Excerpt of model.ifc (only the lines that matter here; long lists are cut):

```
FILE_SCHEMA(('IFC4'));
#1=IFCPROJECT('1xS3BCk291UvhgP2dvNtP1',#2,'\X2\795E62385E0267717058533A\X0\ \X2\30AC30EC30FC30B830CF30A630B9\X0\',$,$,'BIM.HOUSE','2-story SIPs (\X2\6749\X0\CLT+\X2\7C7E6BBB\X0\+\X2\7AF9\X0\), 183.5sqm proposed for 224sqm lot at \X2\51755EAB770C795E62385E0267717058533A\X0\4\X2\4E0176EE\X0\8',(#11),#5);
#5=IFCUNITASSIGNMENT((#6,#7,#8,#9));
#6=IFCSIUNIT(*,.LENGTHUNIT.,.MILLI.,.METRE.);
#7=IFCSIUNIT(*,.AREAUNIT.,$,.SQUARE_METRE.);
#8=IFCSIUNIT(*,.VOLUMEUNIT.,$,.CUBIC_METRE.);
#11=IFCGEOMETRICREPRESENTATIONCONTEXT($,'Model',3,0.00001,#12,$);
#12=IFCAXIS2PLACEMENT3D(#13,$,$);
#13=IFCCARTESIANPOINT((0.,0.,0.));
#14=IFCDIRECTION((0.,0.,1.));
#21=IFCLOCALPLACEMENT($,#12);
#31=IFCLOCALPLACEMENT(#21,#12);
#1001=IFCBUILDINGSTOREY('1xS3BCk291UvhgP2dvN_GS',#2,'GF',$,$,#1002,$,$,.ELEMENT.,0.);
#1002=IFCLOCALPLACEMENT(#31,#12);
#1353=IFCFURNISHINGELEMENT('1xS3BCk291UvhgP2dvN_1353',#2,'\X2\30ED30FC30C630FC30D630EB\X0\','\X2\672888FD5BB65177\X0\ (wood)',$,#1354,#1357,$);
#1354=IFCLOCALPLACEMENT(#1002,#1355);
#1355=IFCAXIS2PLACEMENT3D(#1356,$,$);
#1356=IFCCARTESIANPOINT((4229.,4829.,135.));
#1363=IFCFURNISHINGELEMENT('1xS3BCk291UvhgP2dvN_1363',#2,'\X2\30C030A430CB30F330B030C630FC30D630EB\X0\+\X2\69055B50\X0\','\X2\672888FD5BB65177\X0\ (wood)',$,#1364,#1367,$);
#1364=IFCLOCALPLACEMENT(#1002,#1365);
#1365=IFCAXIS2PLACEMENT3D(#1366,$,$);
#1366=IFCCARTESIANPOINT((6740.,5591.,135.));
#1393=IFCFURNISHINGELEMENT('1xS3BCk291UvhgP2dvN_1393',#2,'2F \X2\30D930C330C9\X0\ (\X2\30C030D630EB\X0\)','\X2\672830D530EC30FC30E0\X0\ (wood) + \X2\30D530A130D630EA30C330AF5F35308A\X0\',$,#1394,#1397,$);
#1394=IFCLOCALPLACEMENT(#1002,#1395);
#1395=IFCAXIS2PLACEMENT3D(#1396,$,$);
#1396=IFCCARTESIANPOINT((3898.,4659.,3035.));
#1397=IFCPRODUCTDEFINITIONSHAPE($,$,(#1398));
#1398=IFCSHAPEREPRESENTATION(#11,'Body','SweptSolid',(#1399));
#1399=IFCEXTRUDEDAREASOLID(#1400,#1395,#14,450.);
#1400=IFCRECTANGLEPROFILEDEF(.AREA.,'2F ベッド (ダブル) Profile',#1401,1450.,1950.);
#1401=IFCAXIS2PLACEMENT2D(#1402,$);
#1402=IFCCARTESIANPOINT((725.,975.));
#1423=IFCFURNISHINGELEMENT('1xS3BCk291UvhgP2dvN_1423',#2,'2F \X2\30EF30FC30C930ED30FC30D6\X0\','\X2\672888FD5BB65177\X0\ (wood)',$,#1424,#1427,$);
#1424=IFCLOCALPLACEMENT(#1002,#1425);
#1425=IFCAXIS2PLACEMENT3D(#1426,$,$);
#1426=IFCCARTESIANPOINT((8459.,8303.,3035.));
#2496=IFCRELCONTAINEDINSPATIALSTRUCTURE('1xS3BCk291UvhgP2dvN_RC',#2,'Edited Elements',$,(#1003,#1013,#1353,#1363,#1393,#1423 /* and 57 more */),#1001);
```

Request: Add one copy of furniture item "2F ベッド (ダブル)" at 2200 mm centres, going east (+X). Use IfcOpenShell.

```python
import numpy as np
import ifcopenshell
import ifcopenshell.api.geometry
import ifcopenshell.api.root
import ifcopenshell.util.element
import ifcopenshell.util.placement

model = ifcopenshell.open("model.ifc")


def reuse_history(source, copy):
    """copy_class also copies each property set's owner history, people and application; keep the originals."""
    for rel in copy.IsDefinedBy:
        if rel.is_a("IfcRelDefinesByProperties") and (history := rel.RelatingPropertyDefinition.OwnerHistory):
            rel.RelatingPropertyDefinition.OwnerHistory = source.OwnerHistory
            ifcopenshell.util.element.remove_deep2(model, history)


source = model.by_guid("1xS3BCk291UvhgP2dvN_1393")
base = ifcopenshell.util.placement.get_local_placement(source.ObjectPlacement)
step = np.array([1.0, 0.0, 0.0]) * 2200.0

for i in range(1, 2):
    copy = ifcopenshell.api.root.copy_class(model, product=source)
    copy.Representation = ifcopenshell.util.element.copy_deep(
        model, source.Representation, exclude=["IfcGeometricRepresentationContext", "IfcRepresentationMap"]
    )
    reuse_history(source, copy)
    matrix = base.copy()
    matrix[:3, 3] += i * step
    print("added at", matrix[:3, 3].round(3) + 0.0)
    ifcopenshell.api.geometry.edit_object_placement(model, product=copy, matrix=matrix, is_si=False)

model.write("model_updated.ifc")
```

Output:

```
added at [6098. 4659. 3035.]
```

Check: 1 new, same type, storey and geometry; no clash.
